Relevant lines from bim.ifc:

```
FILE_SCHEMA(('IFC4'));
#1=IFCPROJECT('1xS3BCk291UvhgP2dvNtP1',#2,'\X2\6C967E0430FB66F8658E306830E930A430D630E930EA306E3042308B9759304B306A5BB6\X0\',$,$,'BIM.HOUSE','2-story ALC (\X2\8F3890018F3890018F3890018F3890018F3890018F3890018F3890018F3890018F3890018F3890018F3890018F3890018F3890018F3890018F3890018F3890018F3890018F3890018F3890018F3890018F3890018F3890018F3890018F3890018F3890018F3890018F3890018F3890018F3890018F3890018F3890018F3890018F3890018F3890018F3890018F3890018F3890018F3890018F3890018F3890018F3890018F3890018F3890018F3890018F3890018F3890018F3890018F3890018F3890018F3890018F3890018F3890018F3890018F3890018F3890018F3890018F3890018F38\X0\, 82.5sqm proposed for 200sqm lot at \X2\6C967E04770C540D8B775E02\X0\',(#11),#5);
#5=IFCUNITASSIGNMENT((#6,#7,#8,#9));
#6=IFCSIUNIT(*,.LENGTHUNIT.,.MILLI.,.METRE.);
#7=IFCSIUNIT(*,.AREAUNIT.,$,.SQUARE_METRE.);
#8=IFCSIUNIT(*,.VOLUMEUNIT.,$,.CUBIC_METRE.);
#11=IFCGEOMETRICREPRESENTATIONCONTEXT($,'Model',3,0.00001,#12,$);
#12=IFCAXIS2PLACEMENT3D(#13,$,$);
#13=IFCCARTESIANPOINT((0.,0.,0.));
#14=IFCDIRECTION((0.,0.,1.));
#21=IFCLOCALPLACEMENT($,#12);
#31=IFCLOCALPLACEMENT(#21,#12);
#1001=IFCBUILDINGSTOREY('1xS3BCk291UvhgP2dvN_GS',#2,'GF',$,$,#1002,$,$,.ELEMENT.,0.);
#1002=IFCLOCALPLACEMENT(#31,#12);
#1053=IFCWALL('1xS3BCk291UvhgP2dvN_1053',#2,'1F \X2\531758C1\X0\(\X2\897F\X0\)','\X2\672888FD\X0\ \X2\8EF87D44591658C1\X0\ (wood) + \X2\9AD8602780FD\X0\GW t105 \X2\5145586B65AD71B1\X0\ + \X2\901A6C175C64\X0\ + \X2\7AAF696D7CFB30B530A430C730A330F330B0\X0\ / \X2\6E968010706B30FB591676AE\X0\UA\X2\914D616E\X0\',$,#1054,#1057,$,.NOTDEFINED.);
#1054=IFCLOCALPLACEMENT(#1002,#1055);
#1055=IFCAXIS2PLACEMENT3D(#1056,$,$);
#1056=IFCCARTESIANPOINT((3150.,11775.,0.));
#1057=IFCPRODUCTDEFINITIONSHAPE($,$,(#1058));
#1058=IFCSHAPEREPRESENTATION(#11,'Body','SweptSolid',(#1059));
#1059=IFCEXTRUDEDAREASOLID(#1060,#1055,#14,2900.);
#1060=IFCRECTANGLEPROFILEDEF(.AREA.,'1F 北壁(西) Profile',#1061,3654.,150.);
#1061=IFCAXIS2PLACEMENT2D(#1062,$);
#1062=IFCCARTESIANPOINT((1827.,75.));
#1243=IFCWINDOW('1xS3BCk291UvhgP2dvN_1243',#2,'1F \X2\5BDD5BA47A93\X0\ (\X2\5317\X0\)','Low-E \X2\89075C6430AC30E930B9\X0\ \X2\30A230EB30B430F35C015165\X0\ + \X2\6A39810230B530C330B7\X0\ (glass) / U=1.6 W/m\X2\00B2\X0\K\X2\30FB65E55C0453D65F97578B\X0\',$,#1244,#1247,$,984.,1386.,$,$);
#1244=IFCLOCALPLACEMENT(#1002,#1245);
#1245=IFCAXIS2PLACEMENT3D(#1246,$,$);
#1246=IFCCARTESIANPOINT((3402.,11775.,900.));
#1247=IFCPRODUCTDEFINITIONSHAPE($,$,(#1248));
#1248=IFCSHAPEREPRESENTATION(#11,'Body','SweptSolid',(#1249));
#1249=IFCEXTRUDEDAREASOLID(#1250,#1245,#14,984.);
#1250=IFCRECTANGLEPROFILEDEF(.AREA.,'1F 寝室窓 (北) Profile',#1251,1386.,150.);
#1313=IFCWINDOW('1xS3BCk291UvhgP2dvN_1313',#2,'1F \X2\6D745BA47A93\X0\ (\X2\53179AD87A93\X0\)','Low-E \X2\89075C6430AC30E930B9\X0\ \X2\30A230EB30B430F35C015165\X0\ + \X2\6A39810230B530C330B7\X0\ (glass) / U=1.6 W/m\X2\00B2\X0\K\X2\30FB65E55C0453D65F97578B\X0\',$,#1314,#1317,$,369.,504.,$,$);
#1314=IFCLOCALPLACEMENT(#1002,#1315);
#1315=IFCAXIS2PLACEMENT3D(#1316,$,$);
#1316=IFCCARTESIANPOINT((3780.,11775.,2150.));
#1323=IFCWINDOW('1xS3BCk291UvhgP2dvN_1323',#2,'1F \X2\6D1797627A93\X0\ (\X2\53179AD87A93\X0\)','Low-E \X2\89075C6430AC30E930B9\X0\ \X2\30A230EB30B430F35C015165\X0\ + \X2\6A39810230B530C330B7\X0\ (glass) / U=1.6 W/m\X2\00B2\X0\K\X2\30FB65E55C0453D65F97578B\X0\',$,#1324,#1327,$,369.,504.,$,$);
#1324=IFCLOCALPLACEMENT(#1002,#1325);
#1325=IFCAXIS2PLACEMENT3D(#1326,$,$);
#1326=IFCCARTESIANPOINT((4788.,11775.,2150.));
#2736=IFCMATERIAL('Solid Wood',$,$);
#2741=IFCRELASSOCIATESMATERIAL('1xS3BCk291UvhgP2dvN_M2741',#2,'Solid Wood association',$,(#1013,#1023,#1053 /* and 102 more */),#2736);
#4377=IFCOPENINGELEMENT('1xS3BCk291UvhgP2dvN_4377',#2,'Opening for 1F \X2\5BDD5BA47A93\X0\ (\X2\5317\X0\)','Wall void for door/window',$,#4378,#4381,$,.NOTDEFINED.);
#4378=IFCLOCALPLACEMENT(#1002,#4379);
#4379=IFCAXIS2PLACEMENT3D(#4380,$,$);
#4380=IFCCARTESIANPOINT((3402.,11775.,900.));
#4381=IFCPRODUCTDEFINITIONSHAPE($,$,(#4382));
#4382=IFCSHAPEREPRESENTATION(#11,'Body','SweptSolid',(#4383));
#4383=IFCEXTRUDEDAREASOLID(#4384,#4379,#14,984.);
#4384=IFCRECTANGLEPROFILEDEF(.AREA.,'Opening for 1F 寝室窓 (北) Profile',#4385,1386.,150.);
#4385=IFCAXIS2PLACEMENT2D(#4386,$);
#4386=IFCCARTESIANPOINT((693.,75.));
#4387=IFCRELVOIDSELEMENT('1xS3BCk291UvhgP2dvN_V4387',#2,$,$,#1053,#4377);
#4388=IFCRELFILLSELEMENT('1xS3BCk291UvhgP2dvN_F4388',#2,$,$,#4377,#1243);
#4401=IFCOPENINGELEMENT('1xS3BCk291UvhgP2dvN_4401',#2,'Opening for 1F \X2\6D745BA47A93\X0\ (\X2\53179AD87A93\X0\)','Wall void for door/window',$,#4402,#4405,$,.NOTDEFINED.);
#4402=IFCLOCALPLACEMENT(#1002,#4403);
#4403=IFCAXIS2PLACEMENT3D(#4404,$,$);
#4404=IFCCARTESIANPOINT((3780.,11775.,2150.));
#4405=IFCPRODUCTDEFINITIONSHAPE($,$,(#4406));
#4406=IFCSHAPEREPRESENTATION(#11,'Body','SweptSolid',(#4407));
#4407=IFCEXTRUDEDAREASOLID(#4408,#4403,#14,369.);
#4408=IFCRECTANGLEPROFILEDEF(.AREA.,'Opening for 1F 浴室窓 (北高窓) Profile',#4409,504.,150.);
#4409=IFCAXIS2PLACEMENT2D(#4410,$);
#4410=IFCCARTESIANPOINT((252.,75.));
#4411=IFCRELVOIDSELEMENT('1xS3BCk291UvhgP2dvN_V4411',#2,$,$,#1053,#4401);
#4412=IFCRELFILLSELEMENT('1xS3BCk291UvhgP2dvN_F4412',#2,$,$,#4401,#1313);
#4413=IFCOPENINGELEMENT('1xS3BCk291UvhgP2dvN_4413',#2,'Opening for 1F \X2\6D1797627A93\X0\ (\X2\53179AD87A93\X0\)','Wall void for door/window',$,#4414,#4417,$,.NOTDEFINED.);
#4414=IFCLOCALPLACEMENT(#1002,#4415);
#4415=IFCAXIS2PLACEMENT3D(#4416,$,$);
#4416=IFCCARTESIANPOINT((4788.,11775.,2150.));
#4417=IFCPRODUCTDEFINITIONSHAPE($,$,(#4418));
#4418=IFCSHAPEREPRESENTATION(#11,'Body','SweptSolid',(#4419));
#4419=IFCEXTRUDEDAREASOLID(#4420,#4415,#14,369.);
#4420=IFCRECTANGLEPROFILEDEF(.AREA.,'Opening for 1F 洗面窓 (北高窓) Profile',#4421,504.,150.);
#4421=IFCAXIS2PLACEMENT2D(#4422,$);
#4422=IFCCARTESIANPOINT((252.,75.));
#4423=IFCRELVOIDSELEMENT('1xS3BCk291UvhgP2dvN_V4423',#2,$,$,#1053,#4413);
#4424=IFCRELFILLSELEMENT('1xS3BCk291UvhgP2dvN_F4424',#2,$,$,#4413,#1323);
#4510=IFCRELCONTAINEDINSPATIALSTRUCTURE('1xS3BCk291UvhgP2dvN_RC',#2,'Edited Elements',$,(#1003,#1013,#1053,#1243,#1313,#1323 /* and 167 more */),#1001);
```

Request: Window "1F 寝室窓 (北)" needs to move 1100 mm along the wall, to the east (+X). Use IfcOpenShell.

```python
import ifcopenshell
import ifcopenshell.api.geometry
import ifcopenshell.util.placement

model = ifcopenshell.open("bim.ifc")

window = model.by_guid("1xS3BCk291UvhgP2dvN_1243")
opening = window.FillsVoids[0].RelatingOpeningElement
wall = opening.VoidsElements[0].RelatingBuildingElement

wall_matrix = ifcopenshell.util.placement.get_local_placement(wall.ObjectPlacement)
shift = wall_matrix[:3, 0] * 1100.0
before = ifcopenshell.util.placement.get_local_placement(window.ObjectPlacement)[:3, 3].copy()

# The window is not placed relative to its opening, so move both.
for product in (opening, window):
    matrix = ifcopenshell.util.placement.get_local_placement(product.ObjectPlacement)
    matrix[:3, 3] += shift
    ifcopenshell.api.geometry.edit_object_placement(model, product=product, matrix=matrix, is_si=False)

after = ifcopenshell.util.placement.get_local_placement(window.ObjectPlacement)[:3, 3]
print("window moved by", (after - before).round(3) + 0.0)

model.write("bim_rev.ifc")
```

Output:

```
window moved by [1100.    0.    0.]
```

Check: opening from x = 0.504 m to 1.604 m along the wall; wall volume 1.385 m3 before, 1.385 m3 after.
